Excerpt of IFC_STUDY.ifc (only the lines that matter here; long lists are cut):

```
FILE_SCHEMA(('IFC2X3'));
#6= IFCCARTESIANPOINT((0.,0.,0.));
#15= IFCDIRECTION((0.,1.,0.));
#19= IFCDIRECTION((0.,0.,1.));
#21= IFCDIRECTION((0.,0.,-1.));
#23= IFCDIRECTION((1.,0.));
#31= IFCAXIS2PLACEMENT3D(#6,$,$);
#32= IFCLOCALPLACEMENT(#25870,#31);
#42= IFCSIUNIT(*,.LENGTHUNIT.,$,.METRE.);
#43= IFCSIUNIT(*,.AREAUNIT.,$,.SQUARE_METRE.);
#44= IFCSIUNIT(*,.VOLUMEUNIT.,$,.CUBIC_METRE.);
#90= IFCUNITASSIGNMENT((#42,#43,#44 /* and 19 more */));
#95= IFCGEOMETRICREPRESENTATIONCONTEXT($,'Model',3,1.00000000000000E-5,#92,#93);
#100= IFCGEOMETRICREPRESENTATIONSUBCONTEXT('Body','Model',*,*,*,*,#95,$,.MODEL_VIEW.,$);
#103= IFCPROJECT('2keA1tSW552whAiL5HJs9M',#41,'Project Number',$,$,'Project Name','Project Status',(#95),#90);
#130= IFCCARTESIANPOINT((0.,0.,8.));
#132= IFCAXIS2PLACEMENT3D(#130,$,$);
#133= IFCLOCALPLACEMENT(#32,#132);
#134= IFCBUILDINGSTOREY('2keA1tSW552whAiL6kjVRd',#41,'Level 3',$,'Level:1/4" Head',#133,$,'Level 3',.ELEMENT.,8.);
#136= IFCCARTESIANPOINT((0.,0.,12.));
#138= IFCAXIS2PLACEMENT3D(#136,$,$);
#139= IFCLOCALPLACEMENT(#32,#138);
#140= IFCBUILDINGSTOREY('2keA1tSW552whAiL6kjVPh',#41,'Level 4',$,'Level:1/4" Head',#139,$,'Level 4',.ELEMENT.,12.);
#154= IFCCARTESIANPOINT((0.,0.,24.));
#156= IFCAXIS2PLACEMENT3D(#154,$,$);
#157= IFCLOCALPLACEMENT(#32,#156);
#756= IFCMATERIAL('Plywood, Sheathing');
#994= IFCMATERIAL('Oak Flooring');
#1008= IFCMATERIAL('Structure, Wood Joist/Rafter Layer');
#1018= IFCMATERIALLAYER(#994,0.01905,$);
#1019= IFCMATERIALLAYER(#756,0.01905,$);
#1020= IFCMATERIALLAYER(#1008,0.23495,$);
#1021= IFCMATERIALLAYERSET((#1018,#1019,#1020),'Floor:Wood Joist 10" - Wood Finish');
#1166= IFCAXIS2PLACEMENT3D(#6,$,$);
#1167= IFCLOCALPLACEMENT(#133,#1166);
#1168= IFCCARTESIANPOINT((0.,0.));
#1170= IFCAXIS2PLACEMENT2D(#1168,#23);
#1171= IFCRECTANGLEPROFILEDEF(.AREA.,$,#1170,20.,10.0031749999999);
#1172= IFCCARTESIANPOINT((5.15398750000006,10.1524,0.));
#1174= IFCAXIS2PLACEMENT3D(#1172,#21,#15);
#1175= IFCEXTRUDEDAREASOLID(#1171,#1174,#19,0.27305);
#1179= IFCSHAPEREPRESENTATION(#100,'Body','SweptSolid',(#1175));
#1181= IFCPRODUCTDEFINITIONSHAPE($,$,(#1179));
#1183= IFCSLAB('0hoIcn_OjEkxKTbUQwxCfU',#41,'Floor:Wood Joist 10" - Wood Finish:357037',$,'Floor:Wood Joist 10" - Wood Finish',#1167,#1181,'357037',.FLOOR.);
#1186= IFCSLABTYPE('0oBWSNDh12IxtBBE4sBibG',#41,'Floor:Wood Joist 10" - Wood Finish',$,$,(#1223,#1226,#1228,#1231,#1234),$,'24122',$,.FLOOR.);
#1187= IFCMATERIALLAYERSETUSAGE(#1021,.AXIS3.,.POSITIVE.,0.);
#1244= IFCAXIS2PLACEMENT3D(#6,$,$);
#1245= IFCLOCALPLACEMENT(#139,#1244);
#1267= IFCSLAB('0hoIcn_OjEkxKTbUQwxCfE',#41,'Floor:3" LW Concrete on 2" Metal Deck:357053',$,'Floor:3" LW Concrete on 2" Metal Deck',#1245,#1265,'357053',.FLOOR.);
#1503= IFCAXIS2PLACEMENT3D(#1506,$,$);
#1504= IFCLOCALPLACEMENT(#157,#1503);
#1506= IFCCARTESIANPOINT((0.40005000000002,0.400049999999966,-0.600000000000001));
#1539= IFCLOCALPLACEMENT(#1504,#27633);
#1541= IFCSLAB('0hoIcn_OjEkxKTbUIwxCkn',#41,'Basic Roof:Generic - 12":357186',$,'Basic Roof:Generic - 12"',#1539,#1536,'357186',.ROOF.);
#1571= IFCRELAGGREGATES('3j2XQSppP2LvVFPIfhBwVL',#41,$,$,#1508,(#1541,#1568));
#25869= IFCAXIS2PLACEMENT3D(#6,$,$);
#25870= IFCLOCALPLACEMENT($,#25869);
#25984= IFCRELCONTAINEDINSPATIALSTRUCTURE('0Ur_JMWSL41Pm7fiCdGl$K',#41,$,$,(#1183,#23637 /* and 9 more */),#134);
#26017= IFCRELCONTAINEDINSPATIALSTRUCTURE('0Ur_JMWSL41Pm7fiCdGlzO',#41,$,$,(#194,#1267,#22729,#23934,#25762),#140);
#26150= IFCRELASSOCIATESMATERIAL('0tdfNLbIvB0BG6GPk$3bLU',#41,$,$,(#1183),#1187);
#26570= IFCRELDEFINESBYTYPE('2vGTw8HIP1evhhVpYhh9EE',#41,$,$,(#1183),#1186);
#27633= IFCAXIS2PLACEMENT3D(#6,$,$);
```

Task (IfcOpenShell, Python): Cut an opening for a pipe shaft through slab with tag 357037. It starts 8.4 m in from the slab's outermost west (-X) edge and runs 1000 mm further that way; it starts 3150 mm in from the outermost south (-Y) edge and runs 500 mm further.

```python
import numpy as np
import ifcopenshell
import ifcopenshell.api.feature
import ifcopenshell.api.geometry
import ifcopenshell.api.root
import ifcopenshell.geom
import ifcopenshell.util.placement
import ifcopenshell.util.representation
import ifcopenshell.util.shape
import ifcopenshell.util.unit

model = ifcopenshell.open("IFC_STUDY.ifc")
unit_scale = ifcopenshell.util.unit.calculate_unit_scale(model)
settings = ifcopenshell.geom.settings()


def volume(element):
    """Net volume in cubic metres, openings subtracted."""
    shape = ifcopenshell.geom.create_shape(settings, element)
    return ifcopenshell.util.shape.get_volume(shape.geometry)


slab = model.by_id(1183)
before = volume(slab)

# Extent in the slab's own axes, in metres. The edges named are its -X and -Y sides.
slab_shape = ifcopenshell.geom.create_shape(settings, slab)
vertices = ifcopenshell.util.shape.get_vertices(slab_shape.geometry)
x_min, y_min, bottom = vertices.min(axis=0)
top = vertices[:, 2].max()

opening = ifcopenshell.api.root.create_entity(model, ifc_class="IfcOpeningElement", name="Pipe shaft opening")
context = ifcopenshell.util.representation.get_context(model, "Model", "Body", "MODEL_VIEW")
width, depth = 1, 0.5
outline = [(0.0, 0.0), (width, 0.0), (width, depth), (0.0, depth), (0.0, 0.0)]
# Overshoot both faces by 50 mm so the cut is clean.
shape = ifcopenshell.api.geometry.add_slab_representation(
    model, context=context, depth=top - bottom + 0.1, polyline=outline
)
ifcopenshell.api.geometry.assign_representation(model, product=opening, representation=shape)

matrix = ifcopenshell.util.placement.get_local_placement(slab.ObjectPlacement)
matrix[:, 3] = matrix @ np.append(np.array([x_min + 8.4, y_min + 3.15, bottom - 0.05]) / unit_scale, 1.0)
ifcopenshell.api.geometry.edit_object_placement(model, product=opening, matrix=matrix, is_si=False)
ifcopenshell.api.feature.add_feature(model, feature=opening, element=slab)

after = volume(slab)

print(f"slab volume {before:.3f} -> {after:.3f} m3")

model.write("IFC_STUDY_edited.ifc")
```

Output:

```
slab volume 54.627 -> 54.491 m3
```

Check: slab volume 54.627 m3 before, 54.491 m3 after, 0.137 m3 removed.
